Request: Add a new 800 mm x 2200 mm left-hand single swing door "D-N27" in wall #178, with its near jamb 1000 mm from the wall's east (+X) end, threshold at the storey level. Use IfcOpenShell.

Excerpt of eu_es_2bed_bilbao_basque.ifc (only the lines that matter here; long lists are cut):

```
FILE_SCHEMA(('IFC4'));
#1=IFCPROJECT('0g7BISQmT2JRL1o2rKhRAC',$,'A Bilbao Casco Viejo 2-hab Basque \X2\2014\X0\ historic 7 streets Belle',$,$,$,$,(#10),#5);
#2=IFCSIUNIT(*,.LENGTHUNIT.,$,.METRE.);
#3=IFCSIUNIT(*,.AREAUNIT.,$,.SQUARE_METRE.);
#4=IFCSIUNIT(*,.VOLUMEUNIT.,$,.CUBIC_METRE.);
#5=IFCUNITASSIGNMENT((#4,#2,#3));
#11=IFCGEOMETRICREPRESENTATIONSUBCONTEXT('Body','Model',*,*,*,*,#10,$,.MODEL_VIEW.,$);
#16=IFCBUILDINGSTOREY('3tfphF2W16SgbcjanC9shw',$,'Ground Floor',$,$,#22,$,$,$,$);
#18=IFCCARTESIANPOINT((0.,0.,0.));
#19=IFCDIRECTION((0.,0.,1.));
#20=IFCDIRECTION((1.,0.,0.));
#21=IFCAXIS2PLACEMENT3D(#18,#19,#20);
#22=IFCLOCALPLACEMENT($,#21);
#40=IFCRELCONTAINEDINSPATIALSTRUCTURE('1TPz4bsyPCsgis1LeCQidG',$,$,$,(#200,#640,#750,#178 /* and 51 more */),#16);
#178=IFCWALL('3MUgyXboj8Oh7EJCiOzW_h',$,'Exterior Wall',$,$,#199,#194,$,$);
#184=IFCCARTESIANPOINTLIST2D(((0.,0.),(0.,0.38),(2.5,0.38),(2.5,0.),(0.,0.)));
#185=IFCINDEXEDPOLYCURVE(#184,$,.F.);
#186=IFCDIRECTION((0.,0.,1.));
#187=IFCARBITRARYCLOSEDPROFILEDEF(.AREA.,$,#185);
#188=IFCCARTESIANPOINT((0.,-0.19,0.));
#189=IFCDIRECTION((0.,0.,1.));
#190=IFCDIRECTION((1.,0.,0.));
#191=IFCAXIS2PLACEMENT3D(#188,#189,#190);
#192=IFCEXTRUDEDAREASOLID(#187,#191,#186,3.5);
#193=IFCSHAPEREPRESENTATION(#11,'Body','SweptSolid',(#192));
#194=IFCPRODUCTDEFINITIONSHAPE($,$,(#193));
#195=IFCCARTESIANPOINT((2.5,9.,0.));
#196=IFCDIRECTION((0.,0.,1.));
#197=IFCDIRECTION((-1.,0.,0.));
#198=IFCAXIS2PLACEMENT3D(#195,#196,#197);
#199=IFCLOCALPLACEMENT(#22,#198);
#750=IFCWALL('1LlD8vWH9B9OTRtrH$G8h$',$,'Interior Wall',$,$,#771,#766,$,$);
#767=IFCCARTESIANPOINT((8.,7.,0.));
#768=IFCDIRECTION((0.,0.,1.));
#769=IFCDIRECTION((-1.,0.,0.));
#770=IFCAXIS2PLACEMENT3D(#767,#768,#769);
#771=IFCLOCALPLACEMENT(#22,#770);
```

```python
import numpy as np
import ifcopenshell
import ifcopenshell.api.feature
import ifcopenshell.api.geometry
import ifcopenshell.api.root
import ifcopenshell.api.spatial
import ifcopenshell.geom
import ifcopenshell.util.element
import ifcopenshell.util.placement
import ifcopenshell.util.representation
import ifcopenshell.util.shape
import ifcopenshell.util.unit

model = ifcopenshell.open("eu_es_2bed_bilbao_basque.ifc")
unit_scale = ifcopenshell.util.unit.calculate_unit_scale(model)
settings = ifcopenshell.geom.settings()


def volume(element):
    """Net volume in cubic metres, openings subtracted."""
    shape = ifcopenshell.geom.create_shape(settings, element)
    return ifcopenshell.util.shape.get_volume(shape.geometry)


wall = model.by_id(178)
storey = ifcopenshell.util.element.get_container(wall, ifc_class="IfcBuildingStorey")
context = ifcopenshell.util.representation.get_context(model, "Model", "Body", "MODEL_VIEW")
before = volume(wall)

width, height, from_end, sill = 0.8, 2.2, 1, 0.0  # metres

# The wall runs along its own X axis, and the end named is its -X end.
wall_shape = ifcopenshell.geom.create_shape(settings, wall)
x, y, z = ifcopenshell.util.shape.get_vertices(wall_shape.geometry).T
start = x.min() + from_end
face, thickness = float(y.min()), float(y.max() - y.min())
wall_matrix = ifcopenshell.util.placement.get_local_placement(wall.ObjectPlacement)
level = ifcopenshell.util.placement.get_local_placement(storey.ObjectPlacement)[2, 3]


def in_wall(x, y):
    """Placement at x, y metres in the wall's axes, at sill height."""
    matrix = wall_matrix.copy()
    matrix[:, 3] = wall_matrix @ np.array([x / unit_scale, y / unit_scale, 0.0, 1.0])
    matrix[2, 3] = level + sill / unit_scale
    return matrix


# Opening: a box that overshoots both wall faces by 50 mm.
opening = ifcopenshell.api.root.create_entity(model, ifc_class="IfcOpeningElement", predefined_type="OPENING")
box = ifcopenshell.api.geometry.add_wall_representation(
    model, context=context, length=width, height=height, thickness=thickness + 0.1
)
ifcopenshell.api.geometry.assign_representation(model, product=opening, representation=box)
ifcopenshell.api.geometry.edit_object_placement(model, product=opening, matrix=in_wall(start, face - 0.05), is_si=False)
ifcopenshell.api.feature.add_feature(model, feature=opening, element=wall)

door = ifcopenshell.api.root.create_entity(model, ifc_class="IfcDoor", name="D-N27", predefined_type="DOOR")
door.OverallWidth, door.OverallHeight = width / unit_scale, height / unit_scale
door.OperationType = "SINGLE_SWING_LEFT"
body = ifcopenshell.api.geometry.add_door_representation(
    model,
    context=context,
    overall_width=door.OverallWidth,
    overall_height=door.OverallHeight,
    operation_type="SINGLE_SWING_LEFT",
    lining_properties={"LiningDepth": thickness / unit_scale, "ThresholdDepth": thickness / unit_scale},
)
ifcopenshell.api.geometry.assign_representation(model, product=door, representation=body)
ifcopenshell.api.spatial.assign_container(model, products=[door], relating_structure=storey)
ifcopenshell.api.feature.add_filling(model, opening=opening, element=door)

# The lining spans the wall, so the door starts at the wall face.
ifcopenshell.api.geometry.edit_object_placement(model, product=door, matrix=in_wall(start, face), is_si=False)

after = volume(wall)

print(f"wall volume {before:.3f} -> {after:.3f} m3")

model.write("eu_es_2bed_bilbao_basque_edited.ifc")
```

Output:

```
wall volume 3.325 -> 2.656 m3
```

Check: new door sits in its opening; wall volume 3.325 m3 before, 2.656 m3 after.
